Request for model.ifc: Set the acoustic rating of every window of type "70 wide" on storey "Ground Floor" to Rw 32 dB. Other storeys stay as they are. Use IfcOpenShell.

First a look at what the model holds.

```python
import ifcopenshell
import ifcopenshell.util.element

model = ifcopenshell.open("model.ifc")
print(model.schema)
storey = next(s for s in model.by_type("IfcBuildingStorey") if s.Name == "Ground Floor")
windows = [e for e in ifcopenshell.util.element.get_decomposition(storey) if e.is_a("IfcWindow")]
seen = {}
for e in windows:
    element_type = ifcopenshell.util.element.get_type(e)
    key = (element_type.Name if element_type != e and element_type else None, ifcopenshell.util.element.get_pset(e, "Pset_WindowCommon", "AcousticRating"))
    seen[key] = seen.get(key, 0) + 1
for (name, value), count in sorted(seen.items(), key=str):
    print(count, "x", name, "|", value)
```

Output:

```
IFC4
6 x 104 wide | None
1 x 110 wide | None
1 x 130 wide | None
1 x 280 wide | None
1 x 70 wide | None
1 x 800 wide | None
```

```python
import ifcopenshell
import ifcopenshell.api.pset
import ifcopenshell.util.element

model = ifcopenshell.open("model.ifc")

storey = next(s for s in model.by_type("IfcBuildingStorey") if s.Name == "Ground Floor")
windows = [e for e in ifcopenshell.util.element.get_decomposition(storey) if e.is_a("IfcWindow")]

count = 0
for e in windows:
    element_type = ifcopenshell.util.element.get_type(e)
    if element_type in (None, e) or element_type.Name != "70 wide":
        continue
    # add_pset returns the element's existing set when there is one.
    pset = ifcopenshell.api.pset.add_pset(model, product=e, name="Pset_WindowCommon")
    ifcopenshell.api.pset.edit_pset(model, pset=pset, properties={"AcousticRating": "Rw 32 dB"})
    count += 1

print(count, "windows updated")

model.write("model_rev.ifc")
```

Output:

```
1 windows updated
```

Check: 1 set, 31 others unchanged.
